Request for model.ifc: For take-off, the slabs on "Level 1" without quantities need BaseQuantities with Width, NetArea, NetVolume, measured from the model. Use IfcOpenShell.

First a look at what the model holds.

```python
import ifcopenshell
import ifcopenshell.util.element
import ifcopenshell.util.unit

model = ifcopenshell.open("model.ifc")
print(model.schema)
for unit_type in ("LENGTHUNIT", "AREAUNIT", "VOLUMEUNIT"):
    print(unit_type, ifcopenshell.util.unit.calculate_unit_scale(model, unit_type))
storey = next(s for s in model.by_type("IfcBuildingStorey") if s.Name == "Level 1")
slabs = [e for e in ifcopenshell.util.element.get_decomposition(storey) if e.is_a("IfcSlab")]
for e in sorted(slabs, key=lambda e: e.id()):
    print(e.id(), e.is_a(), e.Name, list(ifcopenshell.util.element.get_psets(e, qtos_only=True)), sep=" | ")
```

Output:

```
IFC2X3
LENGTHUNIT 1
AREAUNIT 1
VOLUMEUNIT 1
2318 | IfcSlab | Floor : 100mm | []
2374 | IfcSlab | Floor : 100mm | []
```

```python
import ifcopenshell
import ifcopenshell.api.pset
import ifcopenshell.geom
import ifcopenshell.util.element
import ifcopenshell.util.shape
import ifcopenshell.util.unit

model = ifcopenshell.open("model.ifc")
unit_scale = ifcopenshell.util.unit.calculate_unit_scale(model)
area_scale = ifcopenshell.util.unit.calculate_unit_scale(model, "AREAUNIT")
volume_scale = ifcopenshell.util.unit.calculate_unit_scale(model, "VOLUMEUNIT")
settings = ifcopenshell.geom.settings()

storey = next(s for s in model.by_type("IfcBuildingStorey") if s.Name == "Level 1")
slabs = [e for e in ifcopenshell.util.element.get_decomposition(storey) if e.is_a("IfcSlab")]

for e in sorted(slabs, key=lambda e: e.id()):
    if ifcopenshell.util.element.get_psets(e, qtos_only=True, should_inherit=False):
        continue
    # Geometry comes back in metres, in the element's own axes.
    shape = ifcopenshell.geom.create_shape(settings, e)
    values = {
        "Width": ifcopenshell.util.shape.get_z(shape.geometry) / unit_scale,
        "NetArea": ifcopenshell.util.shape.get_footprint_area(shape.geometry) / area_scale,
        "NetVolume": ifcopenshell.util.shape.get_volume(shape.geometry) / volume_scale,
    }
    qto = ifcopenshell.api.pset.add_qto(model, product=e, name="BaseQuantities")
    ifcopenshell.api.pset.edit_qto(model, qto=qto, properties=values)
    print(e.id(), {k: round(v, 3) for k, v in values.items()})

model.write("model_rev.ifc")
```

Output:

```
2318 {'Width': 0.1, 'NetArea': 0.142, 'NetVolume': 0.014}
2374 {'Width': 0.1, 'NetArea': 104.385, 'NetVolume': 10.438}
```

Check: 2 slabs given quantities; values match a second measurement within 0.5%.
